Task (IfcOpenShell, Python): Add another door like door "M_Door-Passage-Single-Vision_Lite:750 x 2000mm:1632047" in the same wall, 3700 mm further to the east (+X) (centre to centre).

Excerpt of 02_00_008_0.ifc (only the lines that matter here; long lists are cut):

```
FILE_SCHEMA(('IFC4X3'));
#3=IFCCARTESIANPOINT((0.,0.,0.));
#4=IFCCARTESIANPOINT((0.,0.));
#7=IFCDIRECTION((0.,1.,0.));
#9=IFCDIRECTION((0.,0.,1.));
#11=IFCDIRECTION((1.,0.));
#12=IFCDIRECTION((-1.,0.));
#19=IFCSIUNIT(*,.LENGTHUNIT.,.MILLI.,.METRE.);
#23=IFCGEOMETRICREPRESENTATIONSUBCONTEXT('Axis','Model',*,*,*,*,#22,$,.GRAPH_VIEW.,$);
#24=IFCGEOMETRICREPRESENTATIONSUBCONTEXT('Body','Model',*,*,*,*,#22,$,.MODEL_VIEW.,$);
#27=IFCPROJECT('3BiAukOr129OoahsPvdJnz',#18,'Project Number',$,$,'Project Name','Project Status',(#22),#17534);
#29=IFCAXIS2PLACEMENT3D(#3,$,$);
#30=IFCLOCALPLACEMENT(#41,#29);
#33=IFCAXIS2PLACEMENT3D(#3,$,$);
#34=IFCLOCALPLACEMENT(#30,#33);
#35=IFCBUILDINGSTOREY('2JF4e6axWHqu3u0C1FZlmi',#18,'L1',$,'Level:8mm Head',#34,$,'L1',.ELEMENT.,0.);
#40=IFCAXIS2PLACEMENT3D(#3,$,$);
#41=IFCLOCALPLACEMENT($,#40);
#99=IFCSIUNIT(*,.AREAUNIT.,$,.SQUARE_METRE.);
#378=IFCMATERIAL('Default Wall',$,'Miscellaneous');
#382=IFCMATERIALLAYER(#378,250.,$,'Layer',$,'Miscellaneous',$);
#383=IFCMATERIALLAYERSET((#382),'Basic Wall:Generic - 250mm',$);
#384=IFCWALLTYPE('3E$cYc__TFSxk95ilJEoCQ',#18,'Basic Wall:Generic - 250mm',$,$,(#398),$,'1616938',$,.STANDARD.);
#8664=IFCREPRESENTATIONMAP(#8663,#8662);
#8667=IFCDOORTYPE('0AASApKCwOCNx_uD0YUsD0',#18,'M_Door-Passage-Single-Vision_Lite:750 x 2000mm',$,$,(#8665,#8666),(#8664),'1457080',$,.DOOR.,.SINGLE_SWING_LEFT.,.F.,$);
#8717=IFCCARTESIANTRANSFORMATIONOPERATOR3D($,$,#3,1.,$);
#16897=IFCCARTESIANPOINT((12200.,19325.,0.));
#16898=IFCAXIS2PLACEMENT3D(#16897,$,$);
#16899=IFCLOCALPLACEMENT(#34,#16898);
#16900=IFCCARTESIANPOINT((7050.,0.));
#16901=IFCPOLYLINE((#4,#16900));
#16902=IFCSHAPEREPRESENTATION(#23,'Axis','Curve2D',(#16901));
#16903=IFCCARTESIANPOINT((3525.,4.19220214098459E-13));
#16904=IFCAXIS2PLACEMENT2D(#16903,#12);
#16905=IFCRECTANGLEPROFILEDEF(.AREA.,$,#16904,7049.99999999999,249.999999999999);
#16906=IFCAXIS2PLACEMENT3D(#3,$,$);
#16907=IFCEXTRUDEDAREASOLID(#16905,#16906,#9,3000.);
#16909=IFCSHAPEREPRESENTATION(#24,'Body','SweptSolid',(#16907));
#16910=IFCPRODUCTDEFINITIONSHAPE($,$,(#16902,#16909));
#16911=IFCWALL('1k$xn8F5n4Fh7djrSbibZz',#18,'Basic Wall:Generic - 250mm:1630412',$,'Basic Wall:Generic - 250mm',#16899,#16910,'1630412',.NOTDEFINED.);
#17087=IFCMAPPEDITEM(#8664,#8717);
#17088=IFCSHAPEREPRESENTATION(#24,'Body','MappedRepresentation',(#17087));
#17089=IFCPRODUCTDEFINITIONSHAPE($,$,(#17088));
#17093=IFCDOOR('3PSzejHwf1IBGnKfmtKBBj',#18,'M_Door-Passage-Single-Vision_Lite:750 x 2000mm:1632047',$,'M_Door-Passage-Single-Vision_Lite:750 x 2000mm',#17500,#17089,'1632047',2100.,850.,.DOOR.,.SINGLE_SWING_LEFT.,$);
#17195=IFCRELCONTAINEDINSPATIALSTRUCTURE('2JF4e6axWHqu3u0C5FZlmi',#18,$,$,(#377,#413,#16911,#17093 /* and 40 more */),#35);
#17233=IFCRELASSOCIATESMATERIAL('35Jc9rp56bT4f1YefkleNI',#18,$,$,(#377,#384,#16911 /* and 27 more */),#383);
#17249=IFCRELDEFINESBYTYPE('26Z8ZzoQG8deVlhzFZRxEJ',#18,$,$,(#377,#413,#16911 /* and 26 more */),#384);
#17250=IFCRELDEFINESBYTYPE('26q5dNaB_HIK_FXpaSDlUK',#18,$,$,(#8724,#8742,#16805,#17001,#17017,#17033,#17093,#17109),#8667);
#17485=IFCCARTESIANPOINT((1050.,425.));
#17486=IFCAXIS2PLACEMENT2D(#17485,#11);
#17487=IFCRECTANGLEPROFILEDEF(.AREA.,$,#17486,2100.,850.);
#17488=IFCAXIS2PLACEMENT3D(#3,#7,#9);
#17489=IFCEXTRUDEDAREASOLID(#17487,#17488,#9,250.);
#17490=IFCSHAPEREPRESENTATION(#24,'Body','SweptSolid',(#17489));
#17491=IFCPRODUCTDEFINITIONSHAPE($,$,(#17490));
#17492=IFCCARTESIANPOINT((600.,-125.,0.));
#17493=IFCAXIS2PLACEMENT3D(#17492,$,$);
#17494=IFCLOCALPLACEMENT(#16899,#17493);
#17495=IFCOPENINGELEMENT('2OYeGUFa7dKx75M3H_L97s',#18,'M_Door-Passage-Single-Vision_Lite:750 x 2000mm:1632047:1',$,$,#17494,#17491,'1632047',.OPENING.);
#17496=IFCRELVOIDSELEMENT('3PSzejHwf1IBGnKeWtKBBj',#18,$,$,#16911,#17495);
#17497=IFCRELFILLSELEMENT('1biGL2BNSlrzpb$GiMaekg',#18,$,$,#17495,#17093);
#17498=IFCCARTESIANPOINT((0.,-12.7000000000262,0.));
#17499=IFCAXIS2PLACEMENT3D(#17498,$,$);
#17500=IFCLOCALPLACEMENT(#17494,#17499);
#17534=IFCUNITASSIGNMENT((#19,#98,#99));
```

```python
import ifcopenshell
import ifcopenshell.api.feature
import ifcopenshell.api.geometry
import ifcopenshell.api.root
import ifcopenshell.geom
import ifcopenshell.util.element
import ifcopenshell.util.placement
import ifcopenshell.util.shape
import ifcopenshell.util.unit

model = ifcopenshell.open("02_00_008_0.ifc")
unit_scale = ifcopenshell.util.unit.calculate_unit_scale(model)
settings = ifcopenshell.geom.settings()


def volume(element):
    """Net volume in cubic metres, openings subtracted."""
    shape = ifcopenshell.geom.create_shape(settings, element)
    return ifcopenshell.util.shape.get_volume(shape.geometry)


def reuse_history(source, copy):
    """copy_class also copies each property set's owner history, people and application; keep the originals."""
    for rel in copy.IsDefinedBy:
        if rel.is_a("IfcRelDefinesByProperties") and (history := rel.RelatingPropertyDefinition.OwnerHistory):
            rel.RelatingPropertyDefinition.OwnerHistory = source.OwnerHistory
            ifcopenshell.util.element.remove_deep2(model, history)


door = model.by_guid("3PSzejHwf1IBGnKfmtKBBj")
opening = door.FillsVoids[0].RelatingOpeningElement
wall = opening.VoidsElements[0].RelatingBuildingElement
before = volume(wall)
shift = ifcopenshell.util.placement.get_local_placement(wall.ObjectPlacement)[:3, 0] * 3.7 / unit_scale

# copy_class copies the void relationship, type, container and properties, but no geometry.
new_opening = ifcopenshell.api.root.copy_class(model, product=opening)
new_opening.Representation = ifcopenshell.util.element.copy_deep(
    model, opening.Representation, exclude=["IfcGeometricRepresentationContext", "IfcRepresentationMap"]
)
new_opening.Name = "M_Door-Passage-Single-Vision_Lite:750 x 2000mm"
new_opening.Tag = None
new_door = ifcopenshell.api.root.copy_class(model, product=door)
new_door.Representation = ifcopenshell.util.element.copy_deep(
    model, door.Representation, exclude=["IfcGeometricRepresentationContext", "IfcRepresentationMap"]
)
new_door.Name = "M_Door-Passage-Single-Vision_Lite:750 x 2000mm"
new_door.Tag = None
reuse_history(door, new_door)
ifcopenshell.api.feature.add_filling(model, opening=new_opening, element=new_door)

for old, new in ((opening, new_opening), (door, new_door)):
    matrix = ifcopenshell.util.placement.get_local_placement(old.ObjectPlacement)
    matrix[:3, 3] += shift
    ifcopenshell.api.geometry.edit_object_placement(model, product=new, matrix=matrix, is_si=False)

after = volume(wall)

print(f"wall volume {before:.3f} -> {after:.3f} m3")

model.write("02_00_008_0_v2.ifc")
```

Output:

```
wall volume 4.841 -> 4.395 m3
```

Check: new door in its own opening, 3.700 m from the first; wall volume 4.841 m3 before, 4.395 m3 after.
